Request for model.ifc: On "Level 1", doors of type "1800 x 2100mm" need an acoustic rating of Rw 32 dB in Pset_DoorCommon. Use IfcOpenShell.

First a look at what the model holds.

```python
import ifcopenshell
import ifcopenshell.util.element

model = ifcopenshell.open("model.ifc")
print(model.schema)
storey = next(s for s in model.by_type("IfcBuildingStorey") if s.Name == "Level 1")
doors = [e for e in ifcopenshell.util.element.get_decomposition(storey) if e.is_a("IfcDoor")]
seen = {}
for e in doors:
    element_type = ifcopenshell.util.element.get_type(e)
    key = (element_type.Name if element_type != e and element_type else None, ifcopenshell.util.element.get_pset(e, "Pset_DoorCommon", "AcousticRating"))
    seen[key] = seen.get(key, 0) + 1
for (name, value), count in sorted(seen.items(), key=str):
    print(count, "x", name, "|", value)
```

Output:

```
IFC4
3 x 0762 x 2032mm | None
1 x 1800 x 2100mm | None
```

```python
import ifcopenshell
import ifcopenshell.api.pset
import ifcopenshell.util.element

model = ifcopenshell.open("model.ifc")

storey = next(s for s in model.by_type("IfcBuildingStorey") if s.Name == "Level 1")
doors = [e for e in ifcopenshell.util.element.get_decomposition(storey) if e.is_a("IfcDoor")]

count = 0
for e in doors:
    element_type = ifcopenshell.util.element.get_type(e)
    if element_type in (None, e) or element_type.Name != "1800 x 2100mm":
        continue
    # add_pset returns the element's existing set when there is one.
    pset = ifcopenshell.api.pset.add_pset(model, product=e, name="Pset_DoorCommon")
    ifcopenshell.api.pset.edit_pset(model, pset=pset, properties={"AcousticRating": "Rw 32 dB"})
    count += 1

print(count, "doors updated")

model.write("model-out.ifc")
```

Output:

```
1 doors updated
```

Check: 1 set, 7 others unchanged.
